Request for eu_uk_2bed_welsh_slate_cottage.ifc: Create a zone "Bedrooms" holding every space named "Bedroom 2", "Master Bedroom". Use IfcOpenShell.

First a look at what the model holds.

```python
import ifcopenshell

model = ifcopenshell.open("eu_uk_2bed_welsh_slate_cottage.ifc")
print(model.schema)
seen = {}
for space in model.by_type("IfcSpace"):
    seen[space.LongName] = seen.get(space.LongName, 0) + 1
for name, count in sorted(seen.items(), key=str):
    print(count, "x", name)
print("zones:", [z.Name for z in model.by_type("IfcZone")][:20])
```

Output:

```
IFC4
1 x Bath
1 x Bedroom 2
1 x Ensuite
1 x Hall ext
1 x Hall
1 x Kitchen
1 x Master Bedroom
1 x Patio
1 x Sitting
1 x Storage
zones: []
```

```python
import ifcopenshell
import ifcopenshell.api.group
import ifcopenshell.api.root

model = ifcopenshell.open("eu_uk_2bed_welsh_slate_cottage.ifc")

names = {"Bedroom 2", "Master Bedroom"}
spaces = [s for s in model.by_type("IfcSpace") if s.LongName in names]

zone = ifcopenshell.api.root.create_entity(model, ifc_class="IfcZone", name="Bedrooms")
ifcopenshell.api.group.assign_group(model, products=spaces, group=zone)
print(len(spaces), "spaces in", zone.Name)

model.write("eu_uk_2bed_welsh_slate_cottage_rev.ifc")
```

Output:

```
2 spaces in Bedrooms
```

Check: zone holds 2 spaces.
